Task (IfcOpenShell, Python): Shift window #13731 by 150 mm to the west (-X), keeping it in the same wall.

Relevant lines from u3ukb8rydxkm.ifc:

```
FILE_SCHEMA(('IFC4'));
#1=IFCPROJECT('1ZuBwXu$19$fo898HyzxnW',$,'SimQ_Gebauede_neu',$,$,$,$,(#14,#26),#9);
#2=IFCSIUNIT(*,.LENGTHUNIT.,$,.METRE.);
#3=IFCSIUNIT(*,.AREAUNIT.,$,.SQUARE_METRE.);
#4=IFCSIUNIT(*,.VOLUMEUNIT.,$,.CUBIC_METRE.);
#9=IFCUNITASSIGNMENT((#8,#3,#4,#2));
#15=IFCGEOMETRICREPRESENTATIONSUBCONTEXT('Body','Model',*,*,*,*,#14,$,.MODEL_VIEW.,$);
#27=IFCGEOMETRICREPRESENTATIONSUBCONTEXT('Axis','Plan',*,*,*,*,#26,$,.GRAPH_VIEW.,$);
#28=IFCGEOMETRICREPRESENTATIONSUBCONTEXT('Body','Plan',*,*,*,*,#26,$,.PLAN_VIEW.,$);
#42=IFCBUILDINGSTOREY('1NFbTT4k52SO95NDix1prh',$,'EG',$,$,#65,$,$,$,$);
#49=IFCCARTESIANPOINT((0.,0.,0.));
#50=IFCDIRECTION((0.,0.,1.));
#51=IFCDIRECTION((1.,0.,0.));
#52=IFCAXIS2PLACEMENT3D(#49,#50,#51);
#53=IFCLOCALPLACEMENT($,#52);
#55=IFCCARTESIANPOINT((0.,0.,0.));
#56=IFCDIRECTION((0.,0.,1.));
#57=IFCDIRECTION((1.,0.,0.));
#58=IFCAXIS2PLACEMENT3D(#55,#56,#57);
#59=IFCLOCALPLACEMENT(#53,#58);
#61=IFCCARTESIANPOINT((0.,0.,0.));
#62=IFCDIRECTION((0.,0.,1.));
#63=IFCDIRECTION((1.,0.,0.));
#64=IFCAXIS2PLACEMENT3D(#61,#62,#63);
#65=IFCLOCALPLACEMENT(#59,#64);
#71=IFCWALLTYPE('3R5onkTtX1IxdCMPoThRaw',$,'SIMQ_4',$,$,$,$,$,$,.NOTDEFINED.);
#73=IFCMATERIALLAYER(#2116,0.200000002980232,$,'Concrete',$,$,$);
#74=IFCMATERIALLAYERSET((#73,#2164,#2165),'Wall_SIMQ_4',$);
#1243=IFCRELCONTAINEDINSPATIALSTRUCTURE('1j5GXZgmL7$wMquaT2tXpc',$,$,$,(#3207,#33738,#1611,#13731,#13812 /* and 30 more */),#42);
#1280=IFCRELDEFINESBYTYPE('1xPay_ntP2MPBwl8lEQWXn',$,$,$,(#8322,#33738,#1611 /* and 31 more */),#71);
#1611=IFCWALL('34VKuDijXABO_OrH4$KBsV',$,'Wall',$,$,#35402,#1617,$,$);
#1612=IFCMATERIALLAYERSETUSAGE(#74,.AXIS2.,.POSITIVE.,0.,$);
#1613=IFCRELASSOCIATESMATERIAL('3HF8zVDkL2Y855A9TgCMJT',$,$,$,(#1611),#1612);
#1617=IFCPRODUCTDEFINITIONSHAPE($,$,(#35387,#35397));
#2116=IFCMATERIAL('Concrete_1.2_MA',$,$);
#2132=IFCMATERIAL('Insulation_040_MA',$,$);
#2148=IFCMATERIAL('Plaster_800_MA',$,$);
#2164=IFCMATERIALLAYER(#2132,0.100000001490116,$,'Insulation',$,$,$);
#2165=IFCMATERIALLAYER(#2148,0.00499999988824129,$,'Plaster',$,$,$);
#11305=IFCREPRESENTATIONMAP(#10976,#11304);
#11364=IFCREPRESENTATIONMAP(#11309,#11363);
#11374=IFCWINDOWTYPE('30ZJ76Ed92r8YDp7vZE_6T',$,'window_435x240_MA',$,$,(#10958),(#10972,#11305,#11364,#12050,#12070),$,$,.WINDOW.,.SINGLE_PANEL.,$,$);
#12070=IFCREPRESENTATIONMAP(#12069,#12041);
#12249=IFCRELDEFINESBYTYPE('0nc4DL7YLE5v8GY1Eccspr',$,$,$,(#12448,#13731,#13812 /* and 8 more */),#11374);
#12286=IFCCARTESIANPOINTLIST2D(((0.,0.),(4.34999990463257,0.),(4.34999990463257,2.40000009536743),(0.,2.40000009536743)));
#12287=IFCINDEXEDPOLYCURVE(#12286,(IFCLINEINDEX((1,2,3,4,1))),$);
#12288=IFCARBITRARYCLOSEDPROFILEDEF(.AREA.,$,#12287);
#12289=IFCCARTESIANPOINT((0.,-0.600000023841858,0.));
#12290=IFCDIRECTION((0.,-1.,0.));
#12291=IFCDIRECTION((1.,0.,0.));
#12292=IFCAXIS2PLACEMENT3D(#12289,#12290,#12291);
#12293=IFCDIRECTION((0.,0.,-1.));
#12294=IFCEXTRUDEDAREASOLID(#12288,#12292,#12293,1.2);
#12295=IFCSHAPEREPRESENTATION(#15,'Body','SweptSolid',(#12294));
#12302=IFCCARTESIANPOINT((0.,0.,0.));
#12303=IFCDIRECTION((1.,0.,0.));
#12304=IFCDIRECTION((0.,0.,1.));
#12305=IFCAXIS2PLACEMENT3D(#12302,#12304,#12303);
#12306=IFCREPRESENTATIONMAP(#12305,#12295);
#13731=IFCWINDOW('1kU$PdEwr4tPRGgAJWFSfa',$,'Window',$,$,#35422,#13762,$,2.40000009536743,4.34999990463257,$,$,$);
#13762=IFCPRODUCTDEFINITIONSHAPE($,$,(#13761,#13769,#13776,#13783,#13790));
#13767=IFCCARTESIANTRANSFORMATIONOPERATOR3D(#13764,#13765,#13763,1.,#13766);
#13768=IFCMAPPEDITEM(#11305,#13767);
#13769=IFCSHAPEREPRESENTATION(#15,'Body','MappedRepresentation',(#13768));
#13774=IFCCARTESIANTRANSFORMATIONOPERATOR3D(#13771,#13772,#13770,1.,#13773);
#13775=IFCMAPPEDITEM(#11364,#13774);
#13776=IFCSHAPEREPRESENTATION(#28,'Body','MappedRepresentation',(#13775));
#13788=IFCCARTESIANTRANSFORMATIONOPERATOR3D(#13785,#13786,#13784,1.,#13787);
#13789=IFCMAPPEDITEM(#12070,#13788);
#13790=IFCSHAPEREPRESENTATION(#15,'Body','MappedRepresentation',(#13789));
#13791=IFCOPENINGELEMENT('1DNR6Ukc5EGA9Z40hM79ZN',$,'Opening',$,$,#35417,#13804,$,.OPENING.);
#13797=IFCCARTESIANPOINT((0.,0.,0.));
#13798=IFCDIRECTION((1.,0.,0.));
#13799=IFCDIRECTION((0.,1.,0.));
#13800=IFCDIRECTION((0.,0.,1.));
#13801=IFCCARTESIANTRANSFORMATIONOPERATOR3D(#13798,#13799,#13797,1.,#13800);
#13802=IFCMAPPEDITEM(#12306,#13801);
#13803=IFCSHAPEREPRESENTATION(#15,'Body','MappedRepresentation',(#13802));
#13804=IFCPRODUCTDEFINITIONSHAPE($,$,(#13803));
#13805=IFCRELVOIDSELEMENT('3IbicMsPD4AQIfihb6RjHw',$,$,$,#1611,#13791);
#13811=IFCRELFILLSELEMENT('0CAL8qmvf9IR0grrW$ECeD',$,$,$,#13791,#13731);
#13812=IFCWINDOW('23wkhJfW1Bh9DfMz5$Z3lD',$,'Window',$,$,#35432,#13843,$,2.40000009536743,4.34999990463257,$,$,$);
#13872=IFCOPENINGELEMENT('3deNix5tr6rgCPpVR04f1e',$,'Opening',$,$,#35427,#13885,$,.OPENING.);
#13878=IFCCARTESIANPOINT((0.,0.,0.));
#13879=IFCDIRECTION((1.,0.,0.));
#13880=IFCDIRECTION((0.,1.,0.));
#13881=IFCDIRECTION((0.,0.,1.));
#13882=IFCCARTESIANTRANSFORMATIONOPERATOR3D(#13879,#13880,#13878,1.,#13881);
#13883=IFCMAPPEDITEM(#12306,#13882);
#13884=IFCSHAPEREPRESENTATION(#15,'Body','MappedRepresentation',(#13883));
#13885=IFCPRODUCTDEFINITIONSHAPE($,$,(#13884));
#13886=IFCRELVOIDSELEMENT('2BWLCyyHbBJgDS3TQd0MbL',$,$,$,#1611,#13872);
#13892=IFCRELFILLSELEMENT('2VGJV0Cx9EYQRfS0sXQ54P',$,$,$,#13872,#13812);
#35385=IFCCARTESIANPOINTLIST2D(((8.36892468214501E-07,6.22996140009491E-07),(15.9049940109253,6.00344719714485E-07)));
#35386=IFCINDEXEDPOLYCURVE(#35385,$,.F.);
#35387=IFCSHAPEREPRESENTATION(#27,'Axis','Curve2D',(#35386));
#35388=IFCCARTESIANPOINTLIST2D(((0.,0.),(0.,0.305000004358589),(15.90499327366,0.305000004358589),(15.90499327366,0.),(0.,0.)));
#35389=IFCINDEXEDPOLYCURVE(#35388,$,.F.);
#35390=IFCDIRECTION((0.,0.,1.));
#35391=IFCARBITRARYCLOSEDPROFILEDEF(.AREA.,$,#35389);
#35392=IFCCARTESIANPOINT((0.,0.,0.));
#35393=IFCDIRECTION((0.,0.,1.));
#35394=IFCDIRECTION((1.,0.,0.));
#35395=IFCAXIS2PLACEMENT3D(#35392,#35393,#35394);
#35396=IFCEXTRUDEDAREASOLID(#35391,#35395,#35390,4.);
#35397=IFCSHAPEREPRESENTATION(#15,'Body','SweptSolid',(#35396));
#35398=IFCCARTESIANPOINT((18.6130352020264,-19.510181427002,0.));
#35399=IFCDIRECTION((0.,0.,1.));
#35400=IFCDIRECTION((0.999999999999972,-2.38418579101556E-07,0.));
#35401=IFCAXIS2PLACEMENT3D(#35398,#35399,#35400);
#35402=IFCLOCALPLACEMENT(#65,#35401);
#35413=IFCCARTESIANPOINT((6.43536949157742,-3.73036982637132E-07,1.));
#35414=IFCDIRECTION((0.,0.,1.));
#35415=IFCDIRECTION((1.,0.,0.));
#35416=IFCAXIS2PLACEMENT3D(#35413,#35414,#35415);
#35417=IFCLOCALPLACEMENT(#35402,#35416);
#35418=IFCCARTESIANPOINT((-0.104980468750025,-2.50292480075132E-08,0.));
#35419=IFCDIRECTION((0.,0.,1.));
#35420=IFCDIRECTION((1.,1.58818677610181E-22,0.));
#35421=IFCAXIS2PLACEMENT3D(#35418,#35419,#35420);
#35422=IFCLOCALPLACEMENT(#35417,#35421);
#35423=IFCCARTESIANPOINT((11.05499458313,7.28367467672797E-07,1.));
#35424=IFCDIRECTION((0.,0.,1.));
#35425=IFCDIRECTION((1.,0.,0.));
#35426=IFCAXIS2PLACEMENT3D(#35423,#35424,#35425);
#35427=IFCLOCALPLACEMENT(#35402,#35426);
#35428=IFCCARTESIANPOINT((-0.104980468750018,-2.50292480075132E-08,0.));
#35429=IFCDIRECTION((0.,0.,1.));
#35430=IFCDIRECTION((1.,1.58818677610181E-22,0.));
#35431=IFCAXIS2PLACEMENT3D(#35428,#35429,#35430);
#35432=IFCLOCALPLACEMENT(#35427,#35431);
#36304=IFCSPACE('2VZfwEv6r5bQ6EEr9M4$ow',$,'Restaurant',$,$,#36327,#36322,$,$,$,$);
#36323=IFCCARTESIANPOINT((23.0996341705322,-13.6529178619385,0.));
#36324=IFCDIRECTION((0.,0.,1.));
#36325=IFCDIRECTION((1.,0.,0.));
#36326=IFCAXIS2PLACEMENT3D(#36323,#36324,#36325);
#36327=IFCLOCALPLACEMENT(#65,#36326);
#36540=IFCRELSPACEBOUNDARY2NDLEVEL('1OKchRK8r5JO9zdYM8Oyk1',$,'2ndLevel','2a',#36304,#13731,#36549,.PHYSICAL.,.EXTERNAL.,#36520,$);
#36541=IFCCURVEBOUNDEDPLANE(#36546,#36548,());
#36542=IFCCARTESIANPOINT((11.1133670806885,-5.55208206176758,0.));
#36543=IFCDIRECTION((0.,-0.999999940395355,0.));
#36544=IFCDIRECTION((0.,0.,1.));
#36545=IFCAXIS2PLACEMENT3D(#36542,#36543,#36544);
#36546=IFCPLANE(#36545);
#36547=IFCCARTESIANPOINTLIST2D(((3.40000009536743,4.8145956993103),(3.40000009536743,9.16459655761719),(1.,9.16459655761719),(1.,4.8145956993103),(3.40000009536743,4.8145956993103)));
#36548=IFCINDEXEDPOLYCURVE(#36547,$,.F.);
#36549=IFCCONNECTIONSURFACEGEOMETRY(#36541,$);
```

```python
import numpy as np
import ifcopenshell
import ifcopenshell.api.geometry
import ifcopenshell.util.placement

model = ifcopenshell.open("u3ukb8rydxkm.ifc")

window = model.by_guid("1kU$PdEwr4tPRGgAJWFSfa")
opening = window.FillsVoids[0].RelatingOpeningElement
wall = opening.VoidsElements[0].RelatingBuildingElement

wall_matrix = ifcopenshell.util.placement.get_local_placement(wall.ObjectPlacement)
shift = wall_matrix[:3, 0] * -0.15
before = ifcopenshell.util.placement.get_local_placement(window.ObjectPlacement)[:3, 3].copy()

# The window is placed relative to its opening, so it follows when the opening moves.
matrix = ifcopenshell.util.placement.get_local_placement(opening.ObjectPlacement)
matrix[:3, 3] += shift
ifcopenshell.api.geometry.edit_object_placement(
    model, product=opening, matrix=matrix, is_si=False, should_transform_children=True
)

# Space boundary surfaces are stored in each space's coordinates; move them too.
for rel in window.ProvidesBoundaries:
    if not rel.ConnectionGeometry:
        continue
    surface = rel.ConnectionGeometry.SurfaceOnRelatingElement.BasisSurface
    space_matrix = ifcopenshell.util.placement.get_local_placement(rel.RelatingSpace.ObjectPlacement)
    point = np.array(surface.Position.Location.Coordinates) + space_matrix[:3, :3].T @ shift
    surface.Position = model.createIfcAxis2Placement3D(
        model.createIfcCartesianPoint(point.tolist()), surface.Position.Axis, surface.Position.RefDirection
    )

after = ifcopenshell.util.placement.get_local_placement(window.ObjectPlacement)[:3, 3]
print("window moved by", (after - before).round(3) + 0.0)

model.write("u3ukb8rydxkm-out.ifc")
```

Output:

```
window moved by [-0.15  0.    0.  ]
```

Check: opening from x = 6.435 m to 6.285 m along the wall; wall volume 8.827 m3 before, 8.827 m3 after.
